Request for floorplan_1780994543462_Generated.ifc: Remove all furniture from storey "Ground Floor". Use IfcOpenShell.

First a look at what the model holds.

```python
import ifcopenshell
import ifcopenshell.util.element

model = ifcopenshell.open("floorplan_1780994543462_Generated.ifc")
print(model.schema)
storey = next(s for s in model.by_type("IfcBuildingStorey") if s.Name == "Ground Floor")
furniture = [e for e in ifcopenshell.util.element.get_decomposition(storey) if e.is_a("IfcFurnishingElement")]
seen = {}
for e in furniture:
    element_type = ifcopenshell.util.element.get_type(e)
    name = element_type.Name if element_type not in (None, e) else None
    seen[name] = seen.get(name, 0) + 1
for name, count in sorted(seen.items(), key=str):
    print(count, "x", name)
```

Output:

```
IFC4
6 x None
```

```python
import ifcopenshell
import ifcopenshell.api.root
import ifcopenshell.util.element

model = ifcopenshell.open("floorplan_1780994543462_Generated.ifc")

storey = next(s for s in model.by_type("IfcBuildingStorey") if s.Name == "Ground Floor")
furniture = [e for e in ifcopenshell.util.element.get_decomposition(storey) if e.is_a("IfcFurnishingElement")]

for e in furniture:
    ifcopenshell.api.root.remove_product(model, product=e)
print(len(furniture), "removed")

model.write("floorplan_1780994543462_Generated_updated.ifc")
```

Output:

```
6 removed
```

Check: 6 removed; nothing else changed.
